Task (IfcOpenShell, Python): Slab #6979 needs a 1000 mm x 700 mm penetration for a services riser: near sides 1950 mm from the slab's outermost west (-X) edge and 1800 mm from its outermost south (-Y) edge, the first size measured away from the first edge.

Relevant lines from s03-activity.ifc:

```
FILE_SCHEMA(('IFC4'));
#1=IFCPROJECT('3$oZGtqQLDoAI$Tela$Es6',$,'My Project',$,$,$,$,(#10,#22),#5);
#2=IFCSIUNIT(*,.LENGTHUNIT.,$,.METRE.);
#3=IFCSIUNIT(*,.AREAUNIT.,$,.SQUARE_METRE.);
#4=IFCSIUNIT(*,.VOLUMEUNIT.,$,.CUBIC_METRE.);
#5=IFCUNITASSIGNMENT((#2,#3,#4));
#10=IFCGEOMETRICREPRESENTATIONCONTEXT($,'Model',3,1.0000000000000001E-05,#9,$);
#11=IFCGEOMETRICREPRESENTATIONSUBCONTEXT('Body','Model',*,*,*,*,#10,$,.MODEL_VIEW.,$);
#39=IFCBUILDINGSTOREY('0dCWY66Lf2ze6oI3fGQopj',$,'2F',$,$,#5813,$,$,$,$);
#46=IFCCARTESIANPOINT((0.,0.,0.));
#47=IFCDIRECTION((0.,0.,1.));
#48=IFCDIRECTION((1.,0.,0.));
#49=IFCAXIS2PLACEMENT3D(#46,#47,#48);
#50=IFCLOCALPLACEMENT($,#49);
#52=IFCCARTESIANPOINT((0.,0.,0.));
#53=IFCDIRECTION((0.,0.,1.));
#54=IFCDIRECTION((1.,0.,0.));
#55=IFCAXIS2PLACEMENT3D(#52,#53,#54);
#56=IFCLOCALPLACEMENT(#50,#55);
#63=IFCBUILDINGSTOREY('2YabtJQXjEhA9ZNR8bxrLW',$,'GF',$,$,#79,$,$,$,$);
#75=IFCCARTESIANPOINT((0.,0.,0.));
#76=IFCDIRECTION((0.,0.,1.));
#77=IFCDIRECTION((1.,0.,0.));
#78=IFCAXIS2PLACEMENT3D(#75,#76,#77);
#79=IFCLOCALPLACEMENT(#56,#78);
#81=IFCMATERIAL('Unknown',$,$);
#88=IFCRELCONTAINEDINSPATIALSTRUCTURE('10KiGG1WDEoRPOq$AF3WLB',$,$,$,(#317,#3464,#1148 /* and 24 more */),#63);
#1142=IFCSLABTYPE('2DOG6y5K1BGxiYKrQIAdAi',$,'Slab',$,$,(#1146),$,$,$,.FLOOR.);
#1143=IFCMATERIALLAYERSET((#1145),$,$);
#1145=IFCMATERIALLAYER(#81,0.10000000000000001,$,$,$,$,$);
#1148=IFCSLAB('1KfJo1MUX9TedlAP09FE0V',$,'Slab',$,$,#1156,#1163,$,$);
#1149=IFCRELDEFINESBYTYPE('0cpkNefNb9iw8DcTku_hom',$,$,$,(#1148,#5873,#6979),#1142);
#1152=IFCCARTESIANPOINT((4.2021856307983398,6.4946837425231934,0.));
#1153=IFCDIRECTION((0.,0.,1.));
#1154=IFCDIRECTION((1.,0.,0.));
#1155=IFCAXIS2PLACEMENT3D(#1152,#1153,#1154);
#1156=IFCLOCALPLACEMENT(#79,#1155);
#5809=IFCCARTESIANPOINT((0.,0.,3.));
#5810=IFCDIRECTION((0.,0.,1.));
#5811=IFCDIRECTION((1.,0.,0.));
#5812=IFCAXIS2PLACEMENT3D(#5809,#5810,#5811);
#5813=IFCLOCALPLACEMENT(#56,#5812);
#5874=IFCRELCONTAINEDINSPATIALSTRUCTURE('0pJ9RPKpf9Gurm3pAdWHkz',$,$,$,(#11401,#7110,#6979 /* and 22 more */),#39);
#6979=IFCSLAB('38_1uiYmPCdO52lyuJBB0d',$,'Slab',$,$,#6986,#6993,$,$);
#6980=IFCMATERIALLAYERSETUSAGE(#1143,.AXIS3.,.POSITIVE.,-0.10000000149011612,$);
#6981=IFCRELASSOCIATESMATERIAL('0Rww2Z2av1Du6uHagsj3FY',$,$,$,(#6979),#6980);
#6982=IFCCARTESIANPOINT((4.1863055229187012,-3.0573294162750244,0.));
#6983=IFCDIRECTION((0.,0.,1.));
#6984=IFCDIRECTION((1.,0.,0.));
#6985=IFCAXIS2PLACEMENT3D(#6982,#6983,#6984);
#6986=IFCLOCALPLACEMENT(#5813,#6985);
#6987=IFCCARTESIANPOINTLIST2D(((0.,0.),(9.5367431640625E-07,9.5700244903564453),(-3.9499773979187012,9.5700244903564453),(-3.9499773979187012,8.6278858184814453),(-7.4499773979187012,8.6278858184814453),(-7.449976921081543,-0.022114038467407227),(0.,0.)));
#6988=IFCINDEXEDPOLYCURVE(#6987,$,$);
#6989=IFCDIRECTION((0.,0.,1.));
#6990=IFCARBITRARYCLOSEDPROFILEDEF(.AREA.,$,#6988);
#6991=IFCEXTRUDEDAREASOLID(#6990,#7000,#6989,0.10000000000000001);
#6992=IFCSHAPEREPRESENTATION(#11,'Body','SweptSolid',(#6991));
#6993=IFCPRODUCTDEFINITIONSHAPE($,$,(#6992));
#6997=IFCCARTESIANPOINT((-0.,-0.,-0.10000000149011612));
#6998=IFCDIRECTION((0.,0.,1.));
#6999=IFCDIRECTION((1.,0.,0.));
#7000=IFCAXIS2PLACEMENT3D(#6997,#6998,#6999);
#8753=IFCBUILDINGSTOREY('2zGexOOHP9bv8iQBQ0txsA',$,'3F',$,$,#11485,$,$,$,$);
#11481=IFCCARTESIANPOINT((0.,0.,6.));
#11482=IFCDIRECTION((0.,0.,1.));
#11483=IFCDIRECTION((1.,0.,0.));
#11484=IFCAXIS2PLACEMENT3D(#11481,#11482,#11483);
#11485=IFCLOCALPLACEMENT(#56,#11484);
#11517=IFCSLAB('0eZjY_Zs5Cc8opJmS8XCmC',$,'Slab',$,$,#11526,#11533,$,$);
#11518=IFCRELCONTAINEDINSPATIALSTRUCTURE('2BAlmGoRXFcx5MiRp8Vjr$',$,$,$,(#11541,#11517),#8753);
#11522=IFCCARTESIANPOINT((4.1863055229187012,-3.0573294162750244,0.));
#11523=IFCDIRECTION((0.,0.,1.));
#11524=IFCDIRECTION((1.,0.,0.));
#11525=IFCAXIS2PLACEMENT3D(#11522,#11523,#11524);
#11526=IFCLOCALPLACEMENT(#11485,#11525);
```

```python
import numpy as np
import ifcopenshell
import ifcopenshell.api.feature
import ifcopenshell.api.geometry
import ifcopenshell.api.root
import ifcopenshell.geom
import ifcopenshell.util.placement
import ifcopenshell.util.representation
import ifcopenshell.util.shape
import ifcopenshell.util.unit

model = ifcopenshell.open("s03-activity.ifc")
unit_scale = ifcopenshell.util.unit.calculate_unit_scale(model)
settings = ifcopenshell.geom.settings()


def volume(element):
    """Net volume in cubic metres, openings subtracted."""
    shape = ifcopenshell.geom.create_shape(settings, element)
    return ifcopenshell.util.shape.get_volume(shape.geometry)


slab = model.by_guid("38_1uiYmPCdO52lyuJBB0d")
before = volume(slab)

# Extent in the slab's own axes, in metres. The edges named are its -X and -Y sides.
slab_shape = ifcopenshell.geom.create_shape(settings, slab)
vertices = ifcopenshell.util.shape.get_vertices(slab_shape.geometry)
x_min, y_min, bottom = vertices.min(axis=0)
top = vertices[:, 2].max()

opening = ifcopenshell.api.root.create_entity(model, ifc_class="IfcOpeningElement", name="Services riser opening", predefined_type="OPENING")
context = ifcopenshell.util.representation.get_context(model, "Model", "Body", "MODEL_VIEW")
width, depth = 1, 0.7
outline = [(0.0, 0.0), (width, 0.0), (width, depth), (0.0, depth), (0.0, 0.0)]
# Overshoot both faces by 50 mm so the cut is clean.
shape = ifcopenshell.api.geometry.add_slab_representation(
    model, context=context, depth=top - bottom + 0.1, polyline=outline
)
ifcopenshell.api.geometry.assign_representation(model, product=opening, representation=shape)

matrix = ifcopenshell.util.placement.get_local_placement(slab.ObjectPlacement)
matrix[:, 3] = matrix @ np.append(np.array([x_min + 1.95, y_min + 1.8, bottom - 0.05]) / unit_scale, 1.0)
ifcopenshell.api.geometry.edit_object_placement(model, product=opening, matrix=matrix, is_si=False)
ifcopenshell.api.feature.add_feature(model, feature=opening, element=slab)

after = volume(slab)

print(f"slab volume {before:.3f} -> {after:.3f} m3")

model.write("s03-activity_edited.ifc")
```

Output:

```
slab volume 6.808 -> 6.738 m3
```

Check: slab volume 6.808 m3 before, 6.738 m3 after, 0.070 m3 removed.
